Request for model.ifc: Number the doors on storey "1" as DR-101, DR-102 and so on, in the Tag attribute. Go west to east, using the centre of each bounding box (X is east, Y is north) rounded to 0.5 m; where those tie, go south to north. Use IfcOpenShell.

First a look at what the model holds.

```python
import ifcopenshell
import ifcopenshell.util.element
import ifcopenshell.util.placement

model = ifcopenshell.open("model.ifc")
print(model.schema)
storey = next(s for s in model.by_type("IfcBuildingStorey") if s.Name == "1")
doors = [e for e in ifcopenshell.util.element.get_decomposition(storey) if e.is_a("IfcDoor")]
for e in sorted(doors, key=lambda e: e.id()):
    origin = ifcopenshell.util.placement.get_local_placement(e.ObjectPlacement)[:3, 3]
    print(e.id(), e.Tag, e.Name, origin.round(2) + 0.0, sep=" | ")
```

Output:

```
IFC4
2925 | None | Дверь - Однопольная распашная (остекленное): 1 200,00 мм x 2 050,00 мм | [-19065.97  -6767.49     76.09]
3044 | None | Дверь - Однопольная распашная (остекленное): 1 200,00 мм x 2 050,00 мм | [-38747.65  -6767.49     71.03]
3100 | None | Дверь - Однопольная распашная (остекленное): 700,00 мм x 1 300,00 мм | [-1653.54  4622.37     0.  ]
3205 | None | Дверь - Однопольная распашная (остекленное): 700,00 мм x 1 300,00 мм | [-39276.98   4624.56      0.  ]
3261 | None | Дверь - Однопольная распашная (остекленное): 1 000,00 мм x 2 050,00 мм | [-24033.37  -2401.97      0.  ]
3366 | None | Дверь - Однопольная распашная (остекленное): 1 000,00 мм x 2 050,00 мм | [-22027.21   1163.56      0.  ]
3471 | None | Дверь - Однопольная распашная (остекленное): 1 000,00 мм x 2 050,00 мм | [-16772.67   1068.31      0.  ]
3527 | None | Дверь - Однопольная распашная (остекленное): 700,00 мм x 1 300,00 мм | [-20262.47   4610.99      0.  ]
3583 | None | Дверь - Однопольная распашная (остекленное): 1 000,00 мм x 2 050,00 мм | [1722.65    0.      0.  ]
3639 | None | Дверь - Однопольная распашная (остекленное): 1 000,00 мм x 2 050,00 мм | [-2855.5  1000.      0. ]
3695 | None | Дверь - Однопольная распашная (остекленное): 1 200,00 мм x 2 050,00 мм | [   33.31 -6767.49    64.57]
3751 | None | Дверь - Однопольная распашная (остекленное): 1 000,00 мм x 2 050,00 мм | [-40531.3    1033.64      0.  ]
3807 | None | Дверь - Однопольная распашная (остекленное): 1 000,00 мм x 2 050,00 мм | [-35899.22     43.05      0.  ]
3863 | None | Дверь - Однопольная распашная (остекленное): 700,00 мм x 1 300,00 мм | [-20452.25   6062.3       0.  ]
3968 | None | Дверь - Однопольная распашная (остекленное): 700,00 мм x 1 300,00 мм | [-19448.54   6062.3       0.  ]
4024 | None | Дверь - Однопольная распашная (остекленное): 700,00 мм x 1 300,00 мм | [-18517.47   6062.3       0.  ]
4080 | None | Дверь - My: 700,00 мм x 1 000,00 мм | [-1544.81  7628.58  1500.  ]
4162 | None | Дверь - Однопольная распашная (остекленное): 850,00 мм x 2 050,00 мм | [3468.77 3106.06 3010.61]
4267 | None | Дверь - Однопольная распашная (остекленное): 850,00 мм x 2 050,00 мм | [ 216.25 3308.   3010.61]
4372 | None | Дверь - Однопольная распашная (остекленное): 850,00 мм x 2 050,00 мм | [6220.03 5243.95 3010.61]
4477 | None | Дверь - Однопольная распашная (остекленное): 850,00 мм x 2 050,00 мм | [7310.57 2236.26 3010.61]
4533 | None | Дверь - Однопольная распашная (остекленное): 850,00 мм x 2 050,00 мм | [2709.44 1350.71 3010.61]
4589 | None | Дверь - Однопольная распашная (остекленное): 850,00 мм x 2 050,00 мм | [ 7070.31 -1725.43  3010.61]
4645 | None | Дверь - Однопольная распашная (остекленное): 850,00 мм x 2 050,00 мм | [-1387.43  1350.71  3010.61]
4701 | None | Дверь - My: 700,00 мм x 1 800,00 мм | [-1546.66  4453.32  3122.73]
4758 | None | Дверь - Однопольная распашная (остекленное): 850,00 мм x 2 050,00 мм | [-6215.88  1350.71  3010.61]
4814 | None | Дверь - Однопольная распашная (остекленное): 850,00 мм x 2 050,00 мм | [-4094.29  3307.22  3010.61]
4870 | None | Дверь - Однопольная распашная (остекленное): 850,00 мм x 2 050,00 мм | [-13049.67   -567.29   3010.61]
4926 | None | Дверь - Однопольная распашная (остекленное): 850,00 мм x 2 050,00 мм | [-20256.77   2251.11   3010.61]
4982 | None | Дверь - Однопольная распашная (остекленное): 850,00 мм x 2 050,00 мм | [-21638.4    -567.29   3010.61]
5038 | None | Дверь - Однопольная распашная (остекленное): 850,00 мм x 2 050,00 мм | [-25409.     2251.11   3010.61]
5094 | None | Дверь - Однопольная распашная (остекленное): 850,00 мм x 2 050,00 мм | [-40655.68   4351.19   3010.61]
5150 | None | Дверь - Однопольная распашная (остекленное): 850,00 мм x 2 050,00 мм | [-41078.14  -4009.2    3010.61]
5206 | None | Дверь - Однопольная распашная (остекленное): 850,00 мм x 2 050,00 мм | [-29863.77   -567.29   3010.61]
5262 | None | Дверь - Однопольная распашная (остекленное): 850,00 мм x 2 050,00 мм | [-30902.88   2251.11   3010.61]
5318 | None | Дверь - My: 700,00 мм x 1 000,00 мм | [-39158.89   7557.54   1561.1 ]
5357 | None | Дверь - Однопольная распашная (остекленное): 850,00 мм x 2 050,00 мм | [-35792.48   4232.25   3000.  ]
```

```python
import ifcopenshell
import ifcopenshell.geom
import ifcopenshell.util.element
import ifcopenshell.util.shape

model = ifcopenshell.open("model.ifc")
settings = ifcopenshell.geom.settings()
settings.set("use-world-coords", True)


def centre(element):
    shape = ifcopenshell.geom.create_shape(settings, element)
    return ifcopenshell.util.shape.get_bbox_centroid(shape.geometry)


storey = next(s for s in model.by_type("IfcBuildingStorey") if s.Name == "1")
doors = [e for e in ifcopenshell.util.element.get_decomposition(storey) if e.is_a("IfcDoor")]

# Insertion points can sit at a corner or the storey origin, so sort by the geometry (in metres).
centres = {e: centre(e) for e in doors}
doors.sort(key=lambda e: (round(centres[e][0] / 0.5), centres[e][1]))

for i, e in enumerate(doors, start=1):
    number = f"DR-1{i:02d}"
    e.Tag = number
    print(e.id(), number)

model.write("model_updated.ifc")
```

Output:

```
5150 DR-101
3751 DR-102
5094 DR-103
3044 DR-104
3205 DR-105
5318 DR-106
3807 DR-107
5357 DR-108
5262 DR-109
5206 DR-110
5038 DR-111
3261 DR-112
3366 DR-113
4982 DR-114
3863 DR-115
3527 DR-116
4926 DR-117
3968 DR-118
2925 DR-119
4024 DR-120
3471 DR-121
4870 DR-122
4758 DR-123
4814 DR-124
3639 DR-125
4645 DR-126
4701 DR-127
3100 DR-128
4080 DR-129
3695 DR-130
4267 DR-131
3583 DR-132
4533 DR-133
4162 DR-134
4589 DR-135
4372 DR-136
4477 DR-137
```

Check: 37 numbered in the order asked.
